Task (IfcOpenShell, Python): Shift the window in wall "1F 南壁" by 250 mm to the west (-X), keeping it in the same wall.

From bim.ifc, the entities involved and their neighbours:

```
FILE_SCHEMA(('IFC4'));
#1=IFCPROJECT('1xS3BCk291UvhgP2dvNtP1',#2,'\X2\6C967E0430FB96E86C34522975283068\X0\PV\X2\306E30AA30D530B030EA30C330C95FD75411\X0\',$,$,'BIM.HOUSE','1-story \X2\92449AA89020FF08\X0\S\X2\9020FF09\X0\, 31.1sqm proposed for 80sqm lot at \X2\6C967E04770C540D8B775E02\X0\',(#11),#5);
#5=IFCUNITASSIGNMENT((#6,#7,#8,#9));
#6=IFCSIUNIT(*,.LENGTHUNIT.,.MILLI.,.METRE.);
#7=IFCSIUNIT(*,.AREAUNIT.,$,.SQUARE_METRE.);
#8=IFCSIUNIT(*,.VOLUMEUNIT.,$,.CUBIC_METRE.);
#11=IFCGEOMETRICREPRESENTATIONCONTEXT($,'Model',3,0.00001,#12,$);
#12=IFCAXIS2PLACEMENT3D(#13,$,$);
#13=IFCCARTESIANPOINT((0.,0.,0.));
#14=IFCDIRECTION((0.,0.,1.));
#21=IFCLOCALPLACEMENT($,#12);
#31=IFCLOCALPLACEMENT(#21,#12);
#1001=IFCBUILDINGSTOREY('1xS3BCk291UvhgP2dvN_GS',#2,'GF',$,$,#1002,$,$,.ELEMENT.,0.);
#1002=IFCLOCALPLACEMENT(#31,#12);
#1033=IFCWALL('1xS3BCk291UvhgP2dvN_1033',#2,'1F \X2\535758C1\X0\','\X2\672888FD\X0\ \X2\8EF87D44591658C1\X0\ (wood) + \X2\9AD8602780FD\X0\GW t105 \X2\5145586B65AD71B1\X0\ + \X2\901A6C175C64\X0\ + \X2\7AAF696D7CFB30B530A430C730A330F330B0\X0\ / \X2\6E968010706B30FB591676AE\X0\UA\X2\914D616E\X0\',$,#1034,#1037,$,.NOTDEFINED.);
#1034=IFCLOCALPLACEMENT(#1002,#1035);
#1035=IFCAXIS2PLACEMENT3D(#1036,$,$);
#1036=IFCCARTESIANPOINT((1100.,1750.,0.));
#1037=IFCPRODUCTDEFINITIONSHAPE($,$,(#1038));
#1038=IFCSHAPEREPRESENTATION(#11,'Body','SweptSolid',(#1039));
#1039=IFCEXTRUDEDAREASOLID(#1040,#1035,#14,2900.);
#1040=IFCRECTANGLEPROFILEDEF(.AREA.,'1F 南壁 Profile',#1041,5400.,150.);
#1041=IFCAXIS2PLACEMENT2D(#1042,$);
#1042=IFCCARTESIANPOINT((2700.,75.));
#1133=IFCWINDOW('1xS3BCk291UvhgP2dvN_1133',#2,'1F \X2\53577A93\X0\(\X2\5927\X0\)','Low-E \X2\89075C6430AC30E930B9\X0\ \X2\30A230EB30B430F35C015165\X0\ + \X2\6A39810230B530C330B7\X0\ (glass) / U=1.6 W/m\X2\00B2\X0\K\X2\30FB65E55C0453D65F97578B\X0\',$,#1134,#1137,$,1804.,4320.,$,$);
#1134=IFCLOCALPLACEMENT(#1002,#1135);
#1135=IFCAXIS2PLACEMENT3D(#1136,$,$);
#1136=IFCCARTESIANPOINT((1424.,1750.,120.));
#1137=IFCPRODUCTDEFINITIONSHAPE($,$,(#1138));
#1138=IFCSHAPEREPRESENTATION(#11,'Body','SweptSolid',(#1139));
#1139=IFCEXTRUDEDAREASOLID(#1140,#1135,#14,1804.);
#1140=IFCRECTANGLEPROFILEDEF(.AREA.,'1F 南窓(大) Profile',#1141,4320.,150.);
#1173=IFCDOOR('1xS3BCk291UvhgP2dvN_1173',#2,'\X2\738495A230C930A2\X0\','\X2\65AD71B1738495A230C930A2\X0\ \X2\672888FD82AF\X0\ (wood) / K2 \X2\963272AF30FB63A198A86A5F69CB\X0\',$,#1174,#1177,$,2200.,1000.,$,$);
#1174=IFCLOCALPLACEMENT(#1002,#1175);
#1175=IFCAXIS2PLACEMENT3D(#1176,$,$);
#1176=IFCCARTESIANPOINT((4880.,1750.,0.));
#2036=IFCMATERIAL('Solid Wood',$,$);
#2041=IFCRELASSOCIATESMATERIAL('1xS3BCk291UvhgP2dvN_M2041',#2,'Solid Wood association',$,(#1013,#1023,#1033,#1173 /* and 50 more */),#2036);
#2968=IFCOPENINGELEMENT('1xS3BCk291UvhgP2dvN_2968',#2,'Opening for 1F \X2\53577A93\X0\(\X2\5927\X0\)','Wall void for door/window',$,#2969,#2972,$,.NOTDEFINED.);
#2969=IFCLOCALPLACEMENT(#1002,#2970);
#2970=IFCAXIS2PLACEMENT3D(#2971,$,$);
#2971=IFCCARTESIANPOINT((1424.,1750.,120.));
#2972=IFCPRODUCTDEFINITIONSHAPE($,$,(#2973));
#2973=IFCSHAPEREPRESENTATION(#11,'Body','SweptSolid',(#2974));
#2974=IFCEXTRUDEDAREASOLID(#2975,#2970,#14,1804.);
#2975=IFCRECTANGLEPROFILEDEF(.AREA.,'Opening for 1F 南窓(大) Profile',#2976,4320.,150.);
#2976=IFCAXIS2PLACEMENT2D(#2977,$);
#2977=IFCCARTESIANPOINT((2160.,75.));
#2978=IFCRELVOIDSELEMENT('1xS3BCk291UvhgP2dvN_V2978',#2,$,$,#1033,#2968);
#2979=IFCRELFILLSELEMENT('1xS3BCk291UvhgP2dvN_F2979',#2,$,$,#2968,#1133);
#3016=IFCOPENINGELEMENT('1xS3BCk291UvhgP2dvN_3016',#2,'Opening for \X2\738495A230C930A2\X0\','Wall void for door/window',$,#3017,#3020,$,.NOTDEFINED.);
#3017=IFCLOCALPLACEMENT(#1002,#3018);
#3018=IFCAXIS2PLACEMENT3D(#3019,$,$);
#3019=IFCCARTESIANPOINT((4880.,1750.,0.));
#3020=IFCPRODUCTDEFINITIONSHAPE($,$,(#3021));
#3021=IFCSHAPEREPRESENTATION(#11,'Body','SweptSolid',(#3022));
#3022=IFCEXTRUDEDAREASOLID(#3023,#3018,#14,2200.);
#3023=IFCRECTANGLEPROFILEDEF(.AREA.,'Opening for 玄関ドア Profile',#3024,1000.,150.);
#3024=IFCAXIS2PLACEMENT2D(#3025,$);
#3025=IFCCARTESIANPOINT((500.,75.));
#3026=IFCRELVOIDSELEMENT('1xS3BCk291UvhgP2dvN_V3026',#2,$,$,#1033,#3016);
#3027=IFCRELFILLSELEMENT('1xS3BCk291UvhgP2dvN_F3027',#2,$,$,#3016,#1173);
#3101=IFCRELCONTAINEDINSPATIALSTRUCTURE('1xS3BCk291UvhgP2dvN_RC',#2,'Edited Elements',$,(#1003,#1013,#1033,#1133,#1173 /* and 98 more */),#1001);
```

```python
import ifcopenshell
import ifcopenshell.api.geometry
import ifcopenshell.util.placement

model = ifcopenshell.open("bim.ifc")

window = model.by_guid("1xS3BCk291UvhgP2dvN_1133")
opening = window.FillsVoids[0].RelatingOpeningElement
wall = opening.VoidsElements[0].RelatingBuildingElement

wall_matrix = ifcopenshell.util.placement.get_local_placement(wall.ObjectPlacement)
shift = wall_matrix[:3, 0] * -250.0
before = ifcopenshell.util.placement.get_local_placement(window.ObjectPlacement)[:3, 3].copy()

# The window is not placed relative to its opening, so move both.
for product in (opening, window):
    matrix = ifcopenshell.util.placement.get_local_placement(product.ObjectPlacement)
    matrix[:3, 3] += shift
    ifcopenshell.api.geometry.edit_object_placement(model, product=product, matrix=matrix, is_si=False)

after = ifcopenshell.util.placement.get_local_placement(window.ObjectPlacement)[:3, 3]
print("window moved by", (after - before).round(3) + 0.0)

model.write("bim_updated.ifc")
```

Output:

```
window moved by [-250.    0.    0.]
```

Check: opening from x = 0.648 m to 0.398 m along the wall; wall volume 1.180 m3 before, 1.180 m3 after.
